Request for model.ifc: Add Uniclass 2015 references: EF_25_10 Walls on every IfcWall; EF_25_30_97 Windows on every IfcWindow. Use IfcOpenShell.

First a look at what the model holds.

```python
import ifcopenshell

model = ifcopenshell.open("model.ifc")
print(model.schema)
print("classifications:", [c.Name for c in model.by_type("IfcClassification")])
for ifc_class in ("IfcDoor", "IfcRoof", "IfcStair", "IfcWall", "IfcWindow"):
    print(ifc_class, len(model.by_type(ifc_class)))
```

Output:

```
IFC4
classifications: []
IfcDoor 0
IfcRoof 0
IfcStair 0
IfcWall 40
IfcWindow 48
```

```python
import ifcopenshell
import ifcopenshell.api.classification

model = ifcopenshell.open("model.ifc")

system = ifcopenshell.api.classification.add_classification(model, classification="Uniclass 2015")

codes = {
    "IfcWall": ("EF_25_10", "Walls"),
    "IfcWindow": ("EF_25_30_97", "Windows"),
}
for ifc_class, (code, name) in codes.items():
    products = model.by_type(ifc_class)
    ifcopenshell.api.classification.add_reference(
        model, products=products, classification=system, identification=code, name=name
    )
    print(code, len(products))

model.write("model_v2.ifc")
```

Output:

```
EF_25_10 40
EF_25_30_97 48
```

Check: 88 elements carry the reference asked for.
